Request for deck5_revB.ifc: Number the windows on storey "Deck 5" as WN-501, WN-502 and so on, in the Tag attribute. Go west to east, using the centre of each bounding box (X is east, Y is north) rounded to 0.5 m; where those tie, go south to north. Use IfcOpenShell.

First a look at what the model holds.

```python
import ifcopenshell
import ifcopenshell.util.element
import ifcopenshell.util.placement

model = ifcopenshell.open("deck5_revB.ifc")
print(model.schema)
storey = next(s for s in model.by_type("IfcBuildingStorey") if s.Name == "Deck 5")
windows = [e for e in ifcopenshell.util.element.get_decomposition(storey) if e.is_a("IfcWindow")]
for e in sorted(windows, key=lambda e: e.id()):
    origin = ifcopenshell.util.placement.get_local_placement(e.ObjectPlacement)[:3, 3]
    print(e.id(), e.Tag, e.Name, origin.round(2) + 0.0, sep=" | ")
```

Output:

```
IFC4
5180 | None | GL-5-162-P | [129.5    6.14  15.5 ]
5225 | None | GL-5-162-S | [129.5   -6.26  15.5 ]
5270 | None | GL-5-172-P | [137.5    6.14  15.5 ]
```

```python
import ifcopenshell
import ifcopenshell.geom
import ifcopenshell.util.element
import ifcopenshell.util.shape

model = ifcopenshell.open("deck5_revB.ifc")
settings = ifcopenshell.geom.settings()
settings.set("use-world-coords", True)


def centre(element):
    shape = ifcopenshell.geom.create_shape(settings, element)
    return ifcopenshell.util.shape.get_bbox_centroid(shape.geometry)


storey = next(s for s in model.by_type("IfcBuildingStorey") if s.Name == "Deck 5")
windows = [e for e in ifcopenshell.util.element.get_decomposition(storey) if e.is_a("IfcWindow")]

# Insertion points can sit at a corner or the storey origin, so sort by the geometry (in metres).
centres = {e: centre(e) for e in windows}
windows.sort(key=lambda e: (round(centres[e][0] / 0.5), centres[e][1]))

for i, e in enumerate(windows, start=1):
    number = f"WN-5{i:02d}"
    e.Tag = number
    print(e.id(), number)

model.write("deck5_revB_rev.ifc")
```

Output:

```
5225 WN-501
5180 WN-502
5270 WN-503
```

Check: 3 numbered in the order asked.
